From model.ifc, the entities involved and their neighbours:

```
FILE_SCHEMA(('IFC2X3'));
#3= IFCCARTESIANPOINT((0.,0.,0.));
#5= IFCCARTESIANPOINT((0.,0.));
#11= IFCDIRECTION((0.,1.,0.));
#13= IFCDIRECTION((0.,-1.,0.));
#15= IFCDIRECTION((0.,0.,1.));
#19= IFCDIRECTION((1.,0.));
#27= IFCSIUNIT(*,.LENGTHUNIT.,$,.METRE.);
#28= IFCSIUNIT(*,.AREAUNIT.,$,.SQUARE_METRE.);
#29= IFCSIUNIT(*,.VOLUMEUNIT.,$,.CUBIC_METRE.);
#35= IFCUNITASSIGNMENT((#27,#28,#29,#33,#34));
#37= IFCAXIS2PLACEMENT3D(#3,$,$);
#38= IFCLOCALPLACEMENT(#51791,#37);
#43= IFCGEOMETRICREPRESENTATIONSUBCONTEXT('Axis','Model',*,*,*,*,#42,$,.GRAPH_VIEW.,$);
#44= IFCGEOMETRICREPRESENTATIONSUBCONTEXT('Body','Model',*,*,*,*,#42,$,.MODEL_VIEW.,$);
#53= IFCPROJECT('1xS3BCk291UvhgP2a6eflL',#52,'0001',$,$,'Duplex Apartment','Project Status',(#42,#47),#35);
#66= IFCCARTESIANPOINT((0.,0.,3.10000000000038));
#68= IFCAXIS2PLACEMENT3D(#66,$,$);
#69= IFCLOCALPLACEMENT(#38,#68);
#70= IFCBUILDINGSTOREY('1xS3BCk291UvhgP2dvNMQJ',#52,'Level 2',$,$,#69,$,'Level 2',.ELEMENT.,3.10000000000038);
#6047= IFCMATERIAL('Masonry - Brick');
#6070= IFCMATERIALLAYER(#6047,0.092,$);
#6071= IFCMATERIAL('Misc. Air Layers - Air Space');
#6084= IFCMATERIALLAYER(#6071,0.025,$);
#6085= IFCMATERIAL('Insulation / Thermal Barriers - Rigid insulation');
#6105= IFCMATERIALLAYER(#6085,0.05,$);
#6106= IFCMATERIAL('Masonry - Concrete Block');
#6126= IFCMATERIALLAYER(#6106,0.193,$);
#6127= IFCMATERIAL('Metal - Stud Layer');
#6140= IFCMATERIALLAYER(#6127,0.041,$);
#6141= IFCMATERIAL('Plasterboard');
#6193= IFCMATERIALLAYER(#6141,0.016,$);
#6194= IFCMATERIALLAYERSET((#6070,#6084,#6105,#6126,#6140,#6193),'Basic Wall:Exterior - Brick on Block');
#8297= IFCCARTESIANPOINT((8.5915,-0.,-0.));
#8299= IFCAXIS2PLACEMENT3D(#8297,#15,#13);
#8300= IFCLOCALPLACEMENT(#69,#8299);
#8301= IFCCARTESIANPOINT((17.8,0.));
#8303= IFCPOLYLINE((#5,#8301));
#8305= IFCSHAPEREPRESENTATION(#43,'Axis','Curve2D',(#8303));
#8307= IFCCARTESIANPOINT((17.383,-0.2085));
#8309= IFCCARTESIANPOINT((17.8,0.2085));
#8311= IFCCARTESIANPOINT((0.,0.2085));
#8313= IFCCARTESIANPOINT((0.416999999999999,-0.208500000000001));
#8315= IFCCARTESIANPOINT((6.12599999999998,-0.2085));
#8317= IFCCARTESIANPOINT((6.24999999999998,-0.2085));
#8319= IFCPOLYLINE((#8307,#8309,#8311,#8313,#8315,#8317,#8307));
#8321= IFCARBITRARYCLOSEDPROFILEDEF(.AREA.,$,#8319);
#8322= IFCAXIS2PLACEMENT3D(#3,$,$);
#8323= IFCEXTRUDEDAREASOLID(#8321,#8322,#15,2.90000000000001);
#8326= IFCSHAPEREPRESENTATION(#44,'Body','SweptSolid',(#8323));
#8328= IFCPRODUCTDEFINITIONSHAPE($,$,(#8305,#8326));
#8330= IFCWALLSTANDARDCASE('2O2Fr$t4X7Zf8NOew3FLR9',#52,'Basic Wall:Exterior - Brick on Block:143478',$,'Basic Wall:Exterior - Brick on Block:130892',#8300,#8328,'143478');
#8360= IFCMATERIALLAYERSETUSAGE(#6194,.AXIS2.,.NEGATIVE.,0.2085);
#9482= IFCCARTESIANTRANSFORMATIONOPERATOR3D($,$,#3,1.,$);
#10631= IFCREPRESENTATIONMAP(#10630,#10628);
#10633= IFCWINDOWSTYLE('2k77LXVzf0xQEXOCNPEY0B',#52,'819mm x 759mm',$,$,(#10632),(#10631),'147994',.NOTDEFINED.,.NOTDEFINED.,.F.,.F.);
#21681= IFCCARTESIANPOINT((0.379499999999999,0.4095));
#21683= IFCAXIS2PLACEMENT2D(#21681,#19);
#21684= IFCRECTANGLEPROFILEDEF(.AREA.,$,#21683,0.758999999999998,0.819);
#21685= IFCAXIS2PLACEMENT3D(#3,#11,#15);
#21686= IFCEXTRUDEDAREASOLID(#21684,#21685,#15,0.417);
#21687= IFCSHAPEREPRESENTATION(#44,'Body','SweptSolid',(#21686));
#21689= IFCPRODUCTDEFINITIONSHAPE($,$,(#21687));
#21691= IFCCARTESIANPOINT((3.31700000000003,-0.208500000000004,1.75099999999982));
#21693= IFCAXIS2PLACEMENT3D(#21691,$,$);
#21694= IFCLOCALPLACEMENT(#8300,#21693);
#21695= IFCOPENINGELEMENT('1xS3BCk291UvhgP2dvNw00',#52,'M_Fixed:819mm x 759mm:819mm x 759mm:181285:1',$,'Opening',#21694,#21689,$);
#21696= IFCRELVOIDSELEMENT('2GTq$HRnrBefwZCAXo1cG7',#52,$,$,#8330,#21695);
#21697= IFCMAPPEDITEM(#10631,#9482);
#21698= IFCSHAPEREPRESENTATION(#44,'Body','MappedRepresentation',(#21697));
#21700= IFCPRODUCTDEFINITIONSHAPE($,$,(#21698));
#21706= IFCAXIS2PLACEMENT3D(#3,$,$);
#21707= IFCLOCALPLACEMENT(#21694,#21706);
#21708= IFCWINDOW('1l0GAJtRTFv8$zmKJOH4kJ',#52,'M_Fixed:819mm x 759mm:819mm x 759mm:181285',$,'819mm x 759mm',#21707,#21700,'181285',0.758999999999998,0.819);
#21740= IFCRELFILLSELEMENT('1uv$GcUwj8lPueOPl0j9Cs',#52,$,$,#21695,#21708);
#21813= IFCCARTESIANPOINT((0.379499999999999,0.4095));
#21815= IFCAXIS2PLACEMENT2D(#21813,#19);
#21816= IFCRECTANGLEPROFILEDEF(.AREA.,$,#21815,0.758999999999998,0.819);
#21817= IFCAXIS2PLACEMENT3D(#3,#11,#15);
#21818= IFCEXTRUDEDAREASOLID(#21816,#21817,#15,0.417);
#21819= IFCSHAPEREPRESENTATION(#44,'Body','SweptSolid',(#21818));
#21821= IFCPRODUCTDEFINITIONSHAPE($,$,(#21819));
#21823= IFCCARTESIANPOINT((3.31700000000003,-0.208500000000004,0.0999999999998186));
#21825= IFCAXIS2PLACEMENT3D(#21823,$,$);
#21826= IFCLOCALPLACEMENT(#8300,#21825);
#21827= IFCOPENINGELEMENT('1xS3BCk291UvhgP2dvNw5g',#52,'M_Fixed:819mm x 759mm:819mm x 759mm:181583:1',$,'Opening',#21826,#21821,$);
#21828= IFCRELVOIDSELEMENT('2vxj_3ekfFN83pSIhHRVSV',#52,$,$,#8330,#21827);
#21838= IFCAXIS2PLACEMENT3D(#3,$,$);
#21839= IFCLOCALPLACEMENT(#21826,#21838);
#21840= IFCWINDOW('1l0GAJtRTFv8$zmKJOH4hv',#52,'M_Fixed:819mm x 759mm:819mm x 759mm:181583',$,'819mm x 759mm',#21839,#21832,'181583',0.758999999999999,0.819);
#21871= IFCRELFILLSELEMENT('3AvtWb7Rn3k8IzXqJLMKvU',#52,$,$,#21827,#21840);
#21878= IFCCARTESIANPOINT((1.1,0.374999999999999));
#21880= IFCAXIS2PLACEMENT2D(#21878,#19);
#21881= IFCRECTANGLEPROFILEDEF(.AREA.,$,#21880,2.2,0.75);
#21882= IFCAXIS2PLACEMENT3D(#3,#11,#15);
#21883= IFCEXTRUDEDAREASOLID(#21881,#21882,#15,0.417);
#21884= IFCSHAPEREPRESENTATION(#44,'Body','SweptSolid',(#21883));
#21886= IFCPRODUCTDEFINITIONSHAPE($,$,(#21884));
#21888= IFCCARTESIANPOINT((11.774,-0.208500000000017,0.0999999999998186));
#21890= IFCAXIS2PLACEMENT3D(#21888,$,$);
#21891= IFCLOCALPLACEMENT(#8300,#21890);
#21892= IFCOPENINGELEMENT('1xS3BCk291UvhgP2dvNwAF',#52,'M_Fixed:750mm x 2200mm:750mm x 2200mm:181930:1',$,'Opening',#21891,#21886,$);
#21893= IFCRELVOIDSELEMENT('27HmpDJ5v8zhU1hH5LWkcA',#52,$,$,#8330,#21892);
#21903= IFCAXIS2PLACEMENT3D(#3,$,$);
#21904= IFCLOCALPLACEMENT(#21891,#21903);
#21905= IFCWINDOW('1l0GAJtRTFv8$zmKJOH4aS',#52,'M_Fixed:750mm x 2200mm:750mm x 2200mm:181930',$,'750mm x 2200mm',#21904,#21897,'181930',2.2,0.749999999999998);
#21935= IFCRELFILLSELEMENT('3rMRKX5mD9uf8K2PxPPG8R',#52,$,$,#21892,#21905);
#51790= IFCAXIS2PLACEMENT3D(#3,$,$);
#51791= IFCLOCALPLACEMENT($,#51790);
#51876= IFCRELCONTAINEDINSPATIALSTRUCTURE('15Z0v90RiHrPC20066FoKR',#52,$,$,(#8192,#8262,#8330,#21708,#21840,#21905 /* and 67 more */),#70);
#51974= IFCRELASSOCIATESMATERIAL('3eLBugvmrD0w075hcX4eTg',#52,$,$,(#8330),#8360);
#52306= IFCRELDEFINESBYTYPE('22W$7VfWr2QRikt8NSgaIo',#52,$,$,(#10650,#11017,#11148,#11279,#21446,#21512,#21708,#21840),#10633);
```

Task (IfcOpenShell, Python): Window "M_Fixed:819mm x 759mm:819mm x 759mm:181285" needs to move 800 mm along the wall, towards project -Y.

```python
import ifcopenshell
import ifcopenshell.api.geometry
import ifcopenshell.util.placement

model = ifcopenshell.open("model.ifc")

window = model.by_guid("1l0GAJtRTFv8$zmKJOH4kJ")
opening = window.FillsVoids[0].RelatingOpeningElement
wall = opening.VoidsElements[0].RelatingBuildingElement

wall_matrix = ifcopenshell.util.placement.get_local_placement(wall.ObjectPlacement)
shift = wall_matrix[:3, 0] * 0.8
before = ifcopenshell.util.placement.get_local_placement(window.ObjectPlacement)[:3, 3].copy()

# The window is placed relative to its opening, so it follows when the opening moves.
matrix = ifcopenshell.util.placement.get_local_placement(opening.ObjectPlacement)
matrix[:3, 3] += shift
ifcopenshell.api.geometry.edit_object_placement(
    model, product=opening, matrix=matrix, is_si=False, should_transform_children=True
)

after = ifcopenshell.util.placement.get_local_placement(window.ObjectPlacement)[:3, 3]
print("window moved by", (after - before).round(3) + 0.0)

model.write("model-out.ifc")
```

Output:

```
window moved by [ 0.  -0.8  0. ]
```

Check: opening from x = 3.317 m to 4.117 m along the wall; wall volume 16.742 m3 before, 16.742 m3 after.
